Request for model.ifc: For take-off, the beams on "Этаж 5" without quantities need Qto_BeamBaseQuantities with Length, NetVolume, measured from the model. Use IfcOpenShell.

First a look at what the model holds.

```python
import ifcopenshell
import ifcopenshell.util.element
import ifcopenshell.util.unit

model = ifcopenshell.open("model.ifc")
print(model.schema)
for unit_type in ("LENGTHUNIT", "AREAUNIT", "VOLUMEUNIT"):
    print(unit_type, ifcopenshell.util.unit.calculate_unit_scale(model, unit_type))
storey = next(s for s in model.by_type("IfcBuildingStorey") if s.Name == "Этаж 5")
beams = [e for e in ifcopenshell.util.element.get_decomposition(storey) if e.is_a("IfcBeam")]
for e in sorted(beams, key=lambda e: e.id()):
    print(e.id(), e.is_a(), e.Name, list(ifcopenshell.util.element.get_psets(e, qtos_only=True)), sep=" | ")
```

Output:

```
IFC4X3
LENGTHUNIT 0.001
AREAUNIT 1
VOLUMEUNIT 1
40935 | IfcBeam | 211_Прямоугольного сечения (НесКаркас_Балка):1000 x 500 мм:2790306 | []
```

```python
import ifcopenshell
import ifcopenshell.api.pset
import ifcopenshell.geom
import ifcopenshell.util.element
import ifcopenshell.util.shape
import ifcopenshell.util.unit

model = ifcopenshell.open("model.ifc")
unit_scale = ifcopenshell.util.unit.calculate_unit_scale(model)
volume_scale = ifcopenshell.util.unit.calculate_unit_scale(model, "VOLUMEUNIT")
settings = ifcopenshell.geom.settings()

storey = next(s for s in model.by_type("IfcBuildingStorey") if s.Name == "Этаж 5")
beams = [e for e in ifcopenshell.util.element.get_decomposition(storey) if e.is_a("IfcBeam")]

for e in sorted(beams, key=lambda e: e.id()):
    if ifcopenshell.util.element.get_psets(e, qtos_only=True, should_inherit=False):
        continue
    # Geometry comes back in metres, in the element's own axes.
    shape = ifcopenshell.geom.create_shape(settings, e)
    values = {
        "Length": ifcopenshell.util.shape.get_max_xyz(shape.geometry) / unit_scale,
        "NetVolume": ifcopenshell.util.shape.get_volume(shape.geometry) / volume_scale,
    }
    qto = ifcopenshell.api.pset.add_qto(model, product=e, name="Qto_BeamBaseQuantities")
    ifcopenshell.api.pset.edit_qto(model, qto=qto, properties=values)
    print(e.id(), {k: round(v, 3) for k, v in values.items()})

model.write("model_updated.ifc")
```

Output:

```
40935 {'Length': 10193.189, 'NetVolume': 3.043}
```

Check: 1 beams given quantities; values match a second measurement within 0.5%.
